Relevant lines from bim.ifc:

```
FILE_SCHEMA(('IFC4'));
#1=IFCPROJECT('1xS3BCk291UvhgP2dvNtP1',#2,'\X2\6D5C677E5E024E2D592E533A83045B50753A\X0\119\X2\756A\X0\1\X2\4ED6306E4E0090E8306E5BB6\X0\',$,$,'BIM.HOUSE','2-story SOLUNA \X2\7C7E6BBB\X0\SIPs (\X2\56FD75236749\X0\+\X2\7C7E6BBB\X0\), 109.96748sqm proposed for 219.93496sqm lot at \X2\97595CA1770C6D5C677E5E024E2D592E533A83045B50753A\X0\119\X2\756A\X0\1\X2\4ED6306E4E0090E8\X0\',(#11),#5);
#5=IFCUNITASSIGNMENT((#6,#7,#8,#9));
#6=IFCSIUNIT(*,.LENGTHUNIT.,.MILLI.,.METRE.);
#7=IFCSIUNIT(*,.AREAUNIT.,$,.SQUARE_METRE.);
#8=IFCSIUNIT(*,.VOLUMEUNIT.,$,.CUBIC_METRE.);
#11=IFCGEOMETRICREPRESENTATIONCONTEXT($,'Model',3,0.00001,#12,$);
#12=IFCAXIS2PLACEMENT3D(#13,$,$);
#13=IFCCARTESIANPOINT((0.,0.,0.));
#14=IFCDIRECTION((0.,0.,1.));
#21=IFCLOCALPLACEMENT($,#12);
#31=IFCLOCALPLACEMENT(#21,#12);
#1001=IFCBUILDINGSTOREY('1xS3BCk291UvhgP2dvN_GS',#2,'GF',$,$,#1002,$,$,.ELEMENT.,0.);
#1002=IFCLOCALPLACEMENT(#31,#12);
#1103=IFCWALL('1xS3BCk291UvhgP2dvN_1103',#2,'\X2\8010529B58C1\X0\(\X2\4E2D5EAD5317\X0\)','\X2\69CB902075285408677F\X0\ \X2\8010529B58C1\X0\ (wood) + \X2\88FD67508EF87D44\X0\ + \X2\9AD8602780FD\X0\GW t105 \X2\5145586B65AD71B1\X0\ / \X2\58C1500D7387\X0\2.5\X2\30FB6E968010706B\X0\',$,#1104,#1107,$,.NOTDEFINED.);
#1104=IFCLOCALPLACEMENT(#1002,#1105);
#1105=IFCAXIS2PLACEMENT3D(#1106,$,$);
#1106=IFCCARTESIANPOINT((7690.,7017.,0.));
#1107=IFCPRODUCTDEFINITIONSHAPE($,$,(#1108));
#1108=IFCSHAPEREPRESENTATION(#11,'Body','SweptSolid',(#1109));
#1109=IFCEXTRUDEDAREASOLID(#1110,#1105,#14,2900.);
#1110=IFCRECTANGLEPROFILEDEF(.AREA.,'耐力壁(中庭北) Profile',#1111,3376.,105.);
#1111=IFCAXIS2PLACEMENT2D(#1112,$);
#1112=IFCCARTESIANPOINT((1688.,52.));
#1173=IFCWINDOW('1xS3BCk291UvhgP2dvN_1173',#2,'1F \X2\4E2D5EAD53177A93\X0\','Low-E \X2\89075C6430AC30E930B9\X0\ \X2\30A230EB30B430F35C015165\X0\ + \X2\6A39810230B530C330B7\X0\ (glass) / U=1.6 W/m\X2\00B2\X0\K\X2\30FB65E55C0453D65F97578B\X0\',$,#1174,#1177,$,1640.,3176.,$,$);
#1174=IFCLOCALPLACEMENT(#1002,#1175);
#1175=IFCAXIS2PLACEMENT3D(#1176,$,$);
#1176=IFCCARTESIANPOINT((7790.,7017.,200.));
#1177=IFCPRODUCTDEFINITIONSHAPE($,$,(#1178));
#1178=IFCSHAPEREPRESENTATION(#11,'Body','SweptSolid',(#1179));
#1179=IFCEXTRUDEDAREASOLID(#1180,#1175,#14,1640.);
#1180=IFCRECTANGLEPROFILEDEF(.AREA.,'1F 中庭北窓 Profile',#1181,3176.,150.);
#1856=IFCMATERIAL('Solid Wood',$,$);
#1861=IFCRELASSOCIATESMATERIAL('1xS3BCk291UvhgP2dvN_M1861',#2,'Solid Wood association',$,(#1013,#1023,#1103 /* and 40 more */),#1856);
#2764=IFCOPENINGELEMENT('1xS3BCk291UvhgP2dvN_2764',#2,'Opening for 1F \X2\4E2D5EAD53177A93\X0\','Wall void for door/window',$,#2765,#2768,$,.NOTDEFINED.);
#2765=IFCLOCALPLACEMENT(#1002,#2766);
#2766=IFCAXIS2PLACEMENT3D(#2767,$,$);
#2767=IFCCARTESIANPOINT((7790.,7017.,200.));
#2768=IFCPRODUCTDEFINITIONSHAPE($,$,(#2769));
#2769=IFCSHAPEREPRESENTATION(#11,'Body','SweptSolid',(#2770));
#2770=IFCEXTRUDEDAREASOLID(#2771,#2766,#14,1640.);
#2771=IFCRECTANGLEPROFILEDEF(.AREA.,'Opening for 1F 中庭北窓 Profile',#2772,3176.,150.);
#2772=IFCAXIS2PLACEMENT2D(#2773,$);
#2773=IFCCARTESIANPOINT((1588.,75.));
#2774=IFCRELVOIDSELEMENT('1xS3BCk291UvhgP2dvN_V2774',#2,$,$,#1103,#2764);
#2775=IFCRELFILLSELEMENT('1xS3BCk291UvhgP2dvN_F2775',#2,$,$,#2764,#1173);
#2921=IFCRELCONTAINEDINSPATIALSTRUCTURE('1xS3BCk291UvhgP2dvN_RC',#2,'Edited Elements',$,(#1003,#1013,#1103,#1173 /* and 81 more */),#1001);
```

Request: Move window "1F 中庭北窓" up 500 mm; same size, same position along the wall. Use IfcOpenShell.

```python
import numpy as np
import ifcopenshell
import ifcopenshell.api.geometry
import ifcopenshell.util.placement
import ifcopenshell.util.unit

model = ifcopenshell.open("bim.ifc")
unit_scale = ifcopenshell.util.unit.calculate_unit_scale(model)

window = model.by_id(1173)
opening = window.FillsVoids[0].RelatingOpeningElement
dz = 0.5 / unit_scale

shift = np.array([0.0, 0.0, dz])
# The window is not placed relative to its opening, so move both.
for product in (opening, window):
    matrix = ifcopenshell.util.placement.get_local_placement(product.ObjectPlacement)
    matrix[:3, 3] += shift
    ifcopenshell.api.geometry.edit_object_placement(model, product=product, matrix=matrix, is_si=False)

print(f"moved by {dz * unit_scale:+.3f} m")

model.write("bim_edited.ifc")
```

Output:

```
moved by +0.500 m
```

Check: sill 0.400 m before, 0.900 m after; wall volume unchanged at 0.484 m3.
